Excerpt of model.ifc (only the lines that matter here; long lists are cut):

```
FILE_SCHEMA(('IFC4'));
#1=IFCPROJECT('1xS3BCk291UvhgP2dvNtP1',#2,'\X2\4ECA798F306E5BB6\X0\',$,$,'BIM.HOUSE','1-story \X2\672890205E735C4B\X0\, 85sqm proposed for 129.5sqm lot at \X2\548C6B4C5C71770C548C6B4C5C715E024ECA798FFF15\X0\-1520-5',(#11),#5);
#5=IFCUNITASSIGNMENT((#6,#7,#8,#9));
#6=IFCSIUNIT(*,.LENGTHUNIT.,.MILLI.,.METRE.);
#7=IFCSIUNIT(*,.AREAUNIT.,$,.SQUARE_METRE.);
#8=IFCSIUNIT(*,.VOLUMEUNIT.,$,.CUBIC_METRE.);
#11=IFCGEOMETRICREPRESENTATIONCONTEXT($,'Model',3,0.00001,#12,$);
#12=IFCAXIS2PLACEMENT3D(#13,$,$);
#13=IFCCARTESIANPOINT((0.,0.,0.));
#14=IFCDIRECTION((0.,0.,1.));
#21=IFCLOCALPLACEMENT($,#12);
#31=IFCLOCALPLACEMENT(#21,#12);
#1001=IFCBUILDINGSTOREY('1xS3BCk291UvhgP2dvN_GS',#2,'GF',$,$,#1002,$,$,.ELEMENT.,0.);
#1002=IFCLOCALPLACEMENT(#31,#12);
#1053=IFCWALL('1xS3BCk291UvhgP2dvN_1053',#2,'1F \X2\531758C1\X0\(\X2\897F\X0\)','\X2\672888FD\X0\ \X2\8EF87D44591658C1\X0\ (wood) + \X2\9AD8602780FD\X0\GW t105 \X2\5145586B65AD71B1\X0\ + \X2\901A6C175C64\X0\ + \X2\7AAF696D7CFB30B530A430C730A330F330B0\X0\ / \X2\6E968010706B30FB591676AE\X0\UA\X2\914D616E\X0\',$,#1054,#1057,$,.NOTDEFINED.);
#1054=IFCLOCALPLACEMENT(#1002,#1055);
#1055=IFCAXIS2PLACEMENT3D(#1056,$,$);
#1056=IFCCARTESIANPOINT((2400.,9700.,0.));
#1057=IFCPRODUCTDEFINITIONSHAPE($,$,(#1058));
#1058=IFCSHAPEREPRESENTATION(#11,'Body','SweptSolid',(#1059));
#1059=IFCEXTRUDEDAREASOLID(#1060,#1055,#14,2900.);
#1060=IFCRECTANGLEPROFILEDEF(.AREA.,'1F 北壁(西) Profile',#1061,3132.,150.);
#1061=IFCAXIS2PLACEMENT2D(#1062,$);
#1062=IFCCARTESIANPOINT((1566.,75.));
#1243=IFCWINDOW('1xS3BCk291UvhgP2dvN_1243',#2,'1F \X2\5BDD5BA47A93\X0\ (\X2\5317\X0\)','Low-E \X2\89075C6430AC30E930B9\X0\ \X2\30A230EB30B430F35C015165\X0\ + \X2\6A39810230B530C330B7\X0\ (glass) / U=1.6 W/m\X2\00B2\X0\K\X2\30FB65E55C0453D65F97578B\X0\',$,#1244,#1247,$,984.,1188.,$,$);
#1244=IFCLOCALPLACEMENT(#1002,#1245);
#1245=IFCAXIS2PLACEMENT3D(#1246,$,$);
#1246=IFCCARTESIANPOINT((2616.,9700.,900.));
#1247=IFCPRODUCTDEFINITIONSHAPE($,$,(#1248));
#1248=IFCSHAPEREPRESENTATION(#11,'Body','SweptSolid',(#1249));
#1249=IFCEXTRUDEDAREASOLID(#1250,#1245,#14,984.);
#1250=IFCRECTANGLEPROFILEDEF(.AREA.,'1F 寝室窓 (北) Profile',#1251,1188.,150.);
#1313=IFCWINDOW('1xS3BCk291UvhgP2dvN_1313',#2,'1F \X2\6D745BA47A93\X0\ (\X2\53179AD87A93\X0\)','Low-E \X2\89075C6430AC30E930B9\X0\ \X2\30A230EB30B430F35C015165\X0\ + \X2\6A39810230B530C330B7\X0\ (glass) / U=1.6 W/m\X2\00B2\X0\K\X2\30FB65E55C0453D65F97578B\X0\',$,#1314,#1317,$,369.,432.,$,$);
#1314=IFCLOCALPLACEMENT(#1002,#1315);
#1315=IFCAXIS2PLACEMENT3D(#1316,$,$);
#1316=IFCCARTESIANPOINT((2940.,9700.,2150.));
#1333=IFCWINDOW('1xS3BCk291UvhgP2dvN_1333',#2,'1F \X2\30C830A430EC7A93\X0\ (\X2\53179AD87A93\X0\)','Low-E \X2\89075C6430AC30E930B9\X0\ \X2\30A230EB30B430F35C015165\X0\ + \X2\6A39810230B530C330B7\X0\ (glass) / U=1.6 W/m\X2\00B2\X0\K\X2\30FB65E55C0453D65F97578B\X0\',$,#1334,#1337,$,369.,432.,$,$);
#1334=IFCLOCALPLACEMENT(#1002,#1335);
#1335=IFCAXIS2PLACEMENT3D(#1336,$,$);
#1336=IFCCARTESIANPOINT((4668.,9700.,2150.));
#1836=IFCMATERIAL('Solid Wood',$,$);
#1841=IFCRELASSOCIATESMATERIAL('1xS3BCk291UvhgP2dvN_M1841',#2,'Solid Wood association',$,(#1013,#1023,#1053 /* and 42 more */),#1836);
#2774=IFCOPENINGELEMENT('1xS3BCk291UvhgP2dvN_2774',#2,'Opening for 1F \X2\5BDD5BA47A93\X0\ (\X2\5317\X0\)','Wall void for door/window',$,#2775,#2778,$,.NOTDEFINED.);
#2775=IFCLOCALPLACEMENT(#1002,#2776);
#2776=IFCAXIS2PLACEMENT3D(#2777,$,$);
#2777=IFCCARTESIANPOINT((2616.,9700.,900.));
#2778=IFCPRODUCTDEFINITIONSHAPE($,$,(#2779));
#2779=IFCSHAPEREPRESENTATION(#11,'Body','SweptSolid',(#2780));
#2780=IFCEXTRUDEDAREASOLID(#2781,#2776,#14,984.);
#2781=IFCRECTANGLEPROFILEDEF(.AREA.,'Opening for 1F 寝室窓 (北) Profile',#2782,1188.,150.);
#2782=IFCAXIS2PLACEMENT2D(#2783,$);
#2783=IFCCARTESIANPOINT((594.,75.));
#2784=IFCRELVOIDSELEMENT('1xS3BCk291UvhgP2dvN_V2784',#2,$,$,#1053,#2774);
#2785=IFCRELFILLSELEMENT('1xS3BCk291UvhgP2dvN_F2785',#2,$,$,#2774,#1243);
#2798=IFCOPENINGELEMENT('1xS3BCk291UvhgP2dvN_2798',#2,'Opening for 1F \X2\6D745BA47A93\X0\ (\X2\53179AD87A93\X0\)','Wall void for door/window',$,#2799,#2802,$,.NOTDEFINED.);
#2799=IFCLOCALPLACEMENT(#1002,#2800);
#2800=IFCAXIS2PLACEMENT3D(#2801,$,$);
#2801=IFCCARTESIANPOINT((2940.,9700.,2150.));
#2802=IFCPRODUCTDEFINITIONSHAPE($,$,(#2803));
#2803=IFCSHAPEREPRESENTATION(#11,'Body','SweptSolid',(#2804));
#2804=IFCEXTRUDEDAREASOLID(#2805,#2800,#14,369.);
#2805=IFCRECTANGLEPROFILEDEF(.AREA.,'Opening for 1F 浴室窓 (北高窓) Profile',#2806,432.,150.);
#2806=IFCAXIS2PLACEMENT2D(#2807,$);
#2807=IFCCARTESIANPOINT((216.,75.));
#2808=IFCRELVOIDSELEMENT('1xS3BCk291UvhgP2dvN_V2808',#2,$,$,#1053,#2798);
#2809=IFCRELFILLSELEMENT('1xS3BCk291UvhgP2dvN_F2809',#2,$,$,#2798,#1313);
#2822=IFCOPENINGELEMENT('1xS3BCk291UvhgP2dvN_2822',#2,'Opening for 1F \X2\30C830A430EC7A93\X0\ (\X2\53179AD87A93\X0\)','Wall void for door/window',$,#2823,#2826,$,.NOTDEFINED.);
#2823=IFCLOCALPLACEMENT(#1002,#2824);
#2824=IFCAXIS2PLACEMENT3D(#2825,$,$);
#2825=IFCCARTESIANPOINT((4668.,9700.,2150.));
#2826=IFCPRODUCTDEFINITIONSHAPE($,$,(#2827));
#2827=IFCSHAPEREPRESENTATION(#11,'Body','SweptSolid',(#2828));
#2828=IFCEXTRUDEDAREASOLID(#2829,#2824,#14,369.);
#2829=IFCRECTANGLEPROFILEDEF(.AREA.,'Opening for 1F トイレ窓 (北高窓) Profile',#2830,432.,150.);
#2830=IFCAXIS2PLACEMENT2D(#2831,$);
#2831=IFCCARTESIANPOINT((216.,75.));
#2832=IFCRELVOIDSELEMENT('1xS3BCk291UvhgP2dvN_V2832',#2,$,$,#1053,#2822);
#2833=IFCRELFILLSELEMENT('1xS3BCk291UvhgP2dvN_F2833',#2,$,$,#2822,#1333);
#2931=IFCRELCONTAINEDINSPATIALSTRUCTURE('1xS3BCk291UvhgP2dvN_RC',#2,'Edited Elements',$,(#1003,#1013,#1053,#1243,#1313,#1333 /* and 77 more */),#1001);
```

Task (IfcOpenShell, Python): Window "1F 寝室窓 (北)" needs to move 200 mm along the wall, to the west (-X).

```python
import ifcopenshell
import ifcopenshell.api.geometry
import ifcopenshell.util.placement
import ifcopenshell.util.unit

model = ifcopenshell.open("model.ifc")
unit_scale = ifcopenshell.util.unit.calculate_unit_scale(model)

window = model.by_guid("1xS3BCk291UvhgP2dvN_1243")
opening = window.FillsVoids[0].RelatingOpeningElement
wall = opening.VoidsElements[0].RelatingBuildingElement

wall_matrix = ifcopenshell.util.placement.get_local_placement(wall.ObjectPlacement)
shift = wall_matrix[:3, 0] * -0.2 / unit_scale
before = ifcopenshell.util.placement.get_local_placement(window.ObjectPlacement)[:3, 3].copy()

# The window is not placed relative to its opening, so move both.
for product in (opening, window):
    matrix = ifcopenshell.util.placement.get_local_placement(product.ObjectPlacement)
    matrix[:3, 3] += shift
    ifcopenshell.api.geometry.edit_object_placement(model, product=product, matrix=matrix, is_si=False)

after = ifcopenshell.util.placement.get_local_placement(window.ObjectPlacement)[:3, 3]
print("window moved by", (after - before).round(3) + 0.0)

model.write("model_updated.ifc")
```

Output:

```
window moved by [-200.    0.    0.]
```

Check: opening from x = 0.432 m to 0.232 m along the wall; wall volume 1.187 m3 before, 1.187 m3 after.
